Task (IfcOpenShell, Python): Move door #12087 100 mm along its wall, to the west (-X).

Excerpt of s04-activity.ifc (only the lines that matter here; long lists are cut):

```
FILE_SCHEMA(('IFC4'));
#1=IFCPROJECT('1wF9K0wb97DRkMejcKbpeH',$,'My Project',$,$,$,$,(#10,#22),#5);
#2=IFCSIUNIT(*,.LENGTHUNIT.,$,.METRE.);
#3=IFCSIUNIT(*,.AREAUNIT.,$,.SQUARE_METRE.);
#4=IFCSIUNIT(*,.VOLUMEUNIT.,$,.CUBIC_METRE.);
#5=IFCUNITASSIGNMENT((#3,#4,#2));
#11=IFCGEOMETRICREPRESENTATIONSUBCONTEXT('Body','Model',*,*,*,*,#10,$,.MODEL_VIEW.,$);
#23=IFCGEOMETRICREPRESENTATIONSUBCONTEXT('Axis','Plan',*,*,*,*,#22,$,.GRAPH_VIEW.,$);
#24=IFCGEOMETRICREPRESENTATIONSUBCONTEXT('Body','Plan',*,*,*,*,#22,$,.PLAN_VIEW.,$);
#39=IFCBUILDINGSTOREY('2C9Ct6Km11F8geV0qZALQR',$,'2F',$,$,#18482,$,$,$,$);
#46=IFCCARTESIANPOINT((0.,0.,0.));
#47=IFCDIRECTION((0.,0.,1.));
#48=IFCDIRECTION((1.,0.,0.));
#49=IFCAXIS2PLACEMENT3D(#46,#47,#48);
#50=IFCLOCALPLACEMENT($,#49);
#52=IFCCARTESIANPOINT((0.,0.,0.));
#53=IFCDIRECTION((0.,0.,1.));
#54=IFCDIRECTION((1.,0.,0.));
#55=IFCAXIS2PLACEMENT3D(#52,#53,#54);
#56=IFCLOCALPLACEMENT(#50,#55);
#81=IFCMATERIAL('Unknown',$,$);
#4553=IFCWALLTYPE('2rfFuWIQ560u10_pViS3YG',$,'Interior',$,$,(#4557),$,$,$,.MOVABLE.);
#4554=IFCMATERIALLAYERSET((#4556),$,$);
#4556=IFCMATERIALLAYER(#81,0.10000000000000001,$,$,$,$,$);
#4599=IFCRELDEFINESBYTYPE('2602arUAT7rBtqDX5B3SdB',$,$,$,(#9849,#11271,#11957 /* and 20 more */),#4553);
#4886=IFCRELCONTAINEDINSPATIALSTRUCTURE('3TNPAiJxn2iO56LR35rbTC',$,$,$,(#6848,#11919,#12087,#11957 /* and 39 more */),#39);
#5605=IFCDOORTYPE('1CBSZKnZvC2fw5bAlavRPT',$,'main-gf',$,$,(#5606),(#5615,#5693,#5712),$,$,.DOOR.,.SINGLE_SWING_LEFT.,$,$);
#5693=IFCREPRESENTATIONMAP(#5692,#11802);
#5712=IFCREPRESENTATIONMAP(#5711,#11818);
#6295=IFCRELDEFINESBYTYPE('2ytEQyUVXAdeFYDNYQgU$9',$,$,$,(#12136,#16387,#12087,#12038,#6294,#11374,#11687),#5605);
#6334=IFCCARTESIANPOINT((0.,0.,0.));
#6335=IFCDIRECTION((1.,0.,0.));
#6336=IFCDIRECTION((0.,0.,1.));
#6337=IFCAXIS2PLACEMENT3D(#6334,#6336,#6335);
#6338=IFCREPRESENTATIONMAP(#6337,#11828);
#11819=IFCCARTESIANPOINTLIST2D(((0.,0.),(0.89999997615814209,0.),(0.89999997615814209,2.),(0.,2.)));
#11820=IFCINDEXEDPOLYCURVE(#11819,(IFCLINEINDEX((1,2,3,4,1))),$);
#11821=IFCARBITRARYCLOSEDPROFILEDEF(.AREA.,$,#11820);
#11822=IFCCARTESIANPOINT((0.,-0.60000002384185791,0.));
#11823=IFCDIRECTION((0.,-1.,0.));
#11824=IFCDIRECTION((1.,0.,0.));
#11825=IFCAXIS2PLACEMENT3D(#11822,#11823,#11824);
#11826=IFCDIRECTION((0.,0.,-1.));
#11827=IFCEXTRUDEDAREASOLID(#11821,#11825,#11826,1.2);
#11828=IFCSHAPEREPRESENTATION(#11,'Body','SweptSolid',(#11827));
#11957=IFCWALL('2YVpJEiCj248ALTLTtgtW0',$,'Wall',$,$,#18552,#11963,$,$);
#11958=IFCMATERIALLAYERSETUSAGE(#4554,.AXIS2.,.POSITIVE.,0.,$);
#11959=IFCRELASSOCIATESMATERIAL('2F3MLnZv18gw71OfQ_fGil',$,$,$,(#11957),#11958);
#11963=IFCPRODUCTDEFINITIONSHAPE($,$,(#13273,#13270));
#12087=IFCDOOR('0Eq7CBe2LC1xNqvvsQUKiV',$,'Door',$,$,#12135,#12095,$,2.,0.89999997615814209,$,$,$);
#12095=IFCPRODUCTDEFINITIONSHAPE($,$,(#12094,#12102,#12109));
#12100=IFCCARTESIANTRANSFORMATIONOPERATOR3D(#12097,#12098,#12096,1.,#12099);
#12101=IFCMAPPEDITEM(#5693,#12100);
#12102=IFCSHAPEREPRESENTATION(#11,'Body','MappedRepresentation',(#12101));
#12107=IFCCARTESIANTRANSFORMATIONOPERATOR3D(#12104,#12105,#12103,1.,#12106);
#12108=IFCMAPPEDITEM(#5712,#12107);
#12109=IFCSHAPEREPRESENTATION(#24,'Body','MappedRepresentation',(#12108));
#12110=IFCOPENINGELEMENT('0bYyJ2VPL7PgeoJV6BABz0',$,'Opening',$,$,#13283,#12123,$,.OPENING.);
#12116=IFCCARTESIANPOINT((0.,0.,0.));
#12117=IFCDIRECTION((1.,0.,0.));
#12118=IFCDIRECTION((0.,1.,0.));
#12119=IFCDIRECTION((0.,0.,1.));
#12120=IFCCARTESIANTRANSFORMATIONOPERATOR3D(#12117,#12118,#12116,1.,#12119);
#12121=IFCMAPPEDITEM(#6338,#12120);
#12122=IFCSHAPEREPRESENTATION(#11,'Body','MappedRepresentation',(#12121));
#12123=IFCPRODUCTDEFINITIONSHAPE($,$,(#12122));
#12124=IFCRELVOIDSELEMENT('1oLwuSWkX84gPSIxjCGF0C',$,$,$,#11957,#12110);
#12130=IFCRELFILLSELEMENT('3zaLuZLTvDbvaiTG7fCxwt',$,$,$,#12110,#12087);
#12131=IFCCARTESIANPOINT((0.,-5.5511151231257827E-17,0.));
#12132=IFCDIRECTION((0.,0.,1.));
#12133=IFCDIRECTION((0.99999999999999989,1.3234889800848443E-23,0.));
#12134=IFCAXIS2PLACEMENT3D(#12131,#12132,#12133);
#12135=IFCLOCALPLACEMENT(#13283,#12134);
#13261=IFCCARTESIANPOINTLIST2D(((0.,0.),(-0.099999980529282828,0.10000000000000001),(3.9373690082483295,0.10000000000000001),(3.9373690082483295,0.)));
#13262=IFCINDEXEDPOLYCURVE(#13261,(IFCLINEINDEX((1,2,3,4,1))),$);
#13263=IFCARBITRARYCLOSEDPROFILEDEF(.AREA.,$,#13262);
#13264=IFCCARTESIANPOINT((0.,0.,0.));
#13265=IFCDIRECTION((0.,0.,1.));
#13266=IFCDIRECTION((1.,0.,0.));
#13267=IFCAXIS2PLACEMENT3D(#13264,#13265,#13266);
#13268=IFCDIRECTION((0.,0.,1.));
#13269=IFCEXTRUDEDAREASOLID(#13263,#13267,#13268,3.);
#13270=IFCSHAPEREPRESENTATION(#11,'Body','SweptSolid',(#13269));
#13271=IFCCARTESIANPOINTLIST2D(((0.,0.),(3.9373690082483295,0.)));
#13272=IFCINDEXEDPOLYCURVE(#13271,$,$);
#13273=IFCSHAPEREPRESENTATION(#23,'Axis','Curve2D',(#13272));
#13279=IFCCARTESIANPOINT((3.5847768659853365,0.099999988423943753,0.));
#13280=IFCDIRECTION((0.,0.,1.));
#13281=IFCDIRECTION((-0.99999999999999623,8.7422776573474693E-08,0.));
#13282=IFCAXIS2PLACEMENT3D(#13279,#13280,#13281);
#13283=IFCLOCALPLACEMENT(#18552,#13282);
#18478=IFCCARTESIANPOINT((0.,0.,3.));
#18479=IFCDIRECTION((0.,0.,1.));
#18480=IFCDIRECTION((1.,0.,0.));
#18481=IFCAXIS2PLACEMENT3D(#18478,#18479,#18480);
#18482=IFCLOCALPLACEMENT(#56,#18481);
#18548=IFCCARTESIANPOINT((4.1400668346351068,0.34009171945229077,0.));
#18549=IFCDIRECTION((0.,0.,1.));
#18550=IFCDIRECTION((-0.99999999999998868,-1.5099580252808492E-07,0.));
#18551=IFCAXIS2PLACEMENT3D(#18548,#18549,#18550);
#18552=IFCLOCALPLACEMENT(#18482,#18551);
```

```python
import ifcopenshell
import ifcopenshell.api.geometry
import ifcopenshell.util.placement

model = ifcopenshell.open("s04-activity.ifc")

door = model.by_guid("0Eq7CBe2LC1xNqvvsQUKiV")
opening = door.FillsVoids[0].RelatingOpeningElement
wall = opening.VoidsElements[0].RelatingBuildingElement

wall_matrix = ifcopenshell.util.placement.get_local_placement(wall.ObjectPlacement)
shift = wall_matrix[:3, 0] * 0.1
before = ifcopenshell.util.placement.get_local_placement(door.ObjectPlacement)[:3, 3].copy()

# The door is placed relative to its opening, so it follows when the opening moves.
matrix = ifcopenshell.util.placement.get_local_placement(opening.ObjectPlacement)
matrix[:3, 3] += shift
ifcopenshell.api.geometry.edit_object_placement(
    model, product=opening, matrix=matrix, is_si=False, should_transform_children=True
)

after = ifcopenshell.util.placement.get_local_placement(door.ObjectPlacement)[:3, 3]
print("door moved by", (after - before).round(3) + 0.0)

model.write("s04-activity_edited.ifc")
```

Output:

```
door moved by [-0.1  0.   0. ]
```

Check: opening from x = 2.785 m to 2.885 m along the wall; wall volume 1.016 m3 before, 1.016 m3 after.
